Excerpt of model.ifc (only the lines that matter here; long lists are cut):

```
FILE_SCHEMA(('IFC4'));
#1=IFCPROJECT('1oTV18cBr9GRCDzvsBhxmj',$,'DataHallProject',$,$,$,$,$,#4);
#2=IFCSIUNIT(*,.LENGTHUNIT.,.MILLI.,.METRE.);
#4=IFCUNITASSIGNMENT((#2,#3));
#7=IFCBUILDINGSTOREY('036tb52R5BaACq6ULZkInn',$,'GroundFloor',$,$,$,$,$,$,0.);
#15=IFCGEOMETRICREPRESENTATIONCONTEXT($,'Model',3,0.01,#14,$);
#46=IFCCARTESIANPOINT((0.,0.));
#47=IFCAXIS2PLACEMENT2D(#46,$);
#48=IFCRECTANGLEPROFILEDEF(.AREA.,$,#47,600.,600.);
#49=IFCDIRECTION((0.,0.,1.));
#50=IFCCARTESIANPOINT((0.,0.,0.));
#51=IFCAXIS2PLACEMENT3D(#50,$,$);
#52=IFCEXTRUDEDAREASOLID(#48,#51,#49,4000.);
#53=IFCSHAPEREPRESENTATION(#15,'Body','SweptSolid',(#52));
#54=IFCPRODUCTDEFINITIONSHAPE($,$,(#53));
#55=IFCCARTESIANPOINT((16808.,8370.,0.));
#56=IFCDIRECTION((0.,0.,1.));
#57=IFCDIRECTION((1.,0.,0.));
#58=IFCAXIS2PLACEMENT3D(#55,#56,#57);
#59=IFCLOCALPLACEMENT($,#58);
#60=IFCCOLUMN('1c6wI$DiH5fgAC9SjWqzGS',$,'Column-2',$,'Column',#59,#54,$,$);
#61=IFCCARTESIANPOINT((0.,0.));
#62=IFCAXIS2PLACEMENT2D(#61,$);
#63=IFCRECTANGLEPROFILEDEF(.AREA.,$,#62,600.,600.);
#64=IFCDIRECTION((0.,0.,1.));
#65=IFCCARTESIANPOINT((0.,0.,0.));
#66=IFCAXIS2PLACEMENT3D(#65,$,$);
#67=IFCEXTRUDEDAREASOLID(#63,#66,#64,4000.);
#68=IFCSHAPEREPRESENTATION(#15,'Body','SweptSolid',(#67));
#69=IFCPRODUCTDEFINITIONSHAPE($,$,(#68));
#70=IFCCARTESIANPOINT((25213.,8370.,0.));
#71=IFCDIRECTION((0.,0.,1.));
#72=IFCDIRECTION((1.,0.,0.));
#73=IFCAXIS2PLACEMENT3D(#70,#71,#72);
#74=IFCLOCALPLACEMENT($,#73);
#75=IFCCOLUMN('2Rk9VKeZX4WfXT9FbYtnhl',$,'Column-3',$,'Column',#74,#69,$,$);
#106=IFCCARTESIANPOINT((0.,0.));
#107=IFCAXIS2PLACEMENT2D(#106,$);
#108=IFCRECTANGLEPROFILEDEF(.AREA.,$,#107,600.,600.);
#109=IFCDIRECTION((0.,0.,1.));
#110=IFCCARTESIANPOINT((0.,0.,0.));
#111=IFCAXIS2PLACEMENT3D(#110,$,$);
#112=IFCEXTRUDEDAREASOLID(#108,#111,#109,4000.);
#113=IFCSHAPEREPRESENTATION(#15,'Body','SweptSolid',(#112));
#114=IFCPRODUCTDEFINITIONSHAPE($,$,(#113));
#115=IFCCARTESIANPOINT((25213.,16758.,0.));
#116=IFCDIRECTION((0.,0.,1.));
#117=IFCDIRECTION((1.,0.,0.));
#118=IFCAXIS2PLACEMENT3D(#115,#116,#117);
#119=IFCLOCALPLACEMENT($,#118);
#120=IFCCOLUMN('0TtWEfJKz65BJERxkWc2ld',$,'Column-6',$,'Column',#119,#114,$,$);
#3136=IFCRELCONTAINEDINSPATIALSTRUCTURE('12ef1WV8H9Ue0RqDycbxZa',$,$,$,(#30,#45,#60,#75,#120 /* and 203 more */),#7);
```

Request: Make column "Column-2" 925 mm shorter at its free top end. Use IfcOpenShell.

```python
import ifcopenshell
import ifcopenshell.util.unit

model = ifcopenshell.open("model.ifc")
unit_scale = ifcopenshell.util.unit.calculate_unit_scale(model)

member = model.by_guid("1c6wI$DiH5fgAC9SjWqzGS")
change = -0.925 / unit_scale

# The extrusion runs towards the end named, so only its depth changes.
body = next(r for r in member.Representation.Representations if r.RepresentationIdentifier == "Body")
solid = body.Items[0]
old_length = solid.Depth
solid.Depth += change

print(f"length {old_length:g} -> {solid.Depth:g}")

model.write("model-out.ifc")
```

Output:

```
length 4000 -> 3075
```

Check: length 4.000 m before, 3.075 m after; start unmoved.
